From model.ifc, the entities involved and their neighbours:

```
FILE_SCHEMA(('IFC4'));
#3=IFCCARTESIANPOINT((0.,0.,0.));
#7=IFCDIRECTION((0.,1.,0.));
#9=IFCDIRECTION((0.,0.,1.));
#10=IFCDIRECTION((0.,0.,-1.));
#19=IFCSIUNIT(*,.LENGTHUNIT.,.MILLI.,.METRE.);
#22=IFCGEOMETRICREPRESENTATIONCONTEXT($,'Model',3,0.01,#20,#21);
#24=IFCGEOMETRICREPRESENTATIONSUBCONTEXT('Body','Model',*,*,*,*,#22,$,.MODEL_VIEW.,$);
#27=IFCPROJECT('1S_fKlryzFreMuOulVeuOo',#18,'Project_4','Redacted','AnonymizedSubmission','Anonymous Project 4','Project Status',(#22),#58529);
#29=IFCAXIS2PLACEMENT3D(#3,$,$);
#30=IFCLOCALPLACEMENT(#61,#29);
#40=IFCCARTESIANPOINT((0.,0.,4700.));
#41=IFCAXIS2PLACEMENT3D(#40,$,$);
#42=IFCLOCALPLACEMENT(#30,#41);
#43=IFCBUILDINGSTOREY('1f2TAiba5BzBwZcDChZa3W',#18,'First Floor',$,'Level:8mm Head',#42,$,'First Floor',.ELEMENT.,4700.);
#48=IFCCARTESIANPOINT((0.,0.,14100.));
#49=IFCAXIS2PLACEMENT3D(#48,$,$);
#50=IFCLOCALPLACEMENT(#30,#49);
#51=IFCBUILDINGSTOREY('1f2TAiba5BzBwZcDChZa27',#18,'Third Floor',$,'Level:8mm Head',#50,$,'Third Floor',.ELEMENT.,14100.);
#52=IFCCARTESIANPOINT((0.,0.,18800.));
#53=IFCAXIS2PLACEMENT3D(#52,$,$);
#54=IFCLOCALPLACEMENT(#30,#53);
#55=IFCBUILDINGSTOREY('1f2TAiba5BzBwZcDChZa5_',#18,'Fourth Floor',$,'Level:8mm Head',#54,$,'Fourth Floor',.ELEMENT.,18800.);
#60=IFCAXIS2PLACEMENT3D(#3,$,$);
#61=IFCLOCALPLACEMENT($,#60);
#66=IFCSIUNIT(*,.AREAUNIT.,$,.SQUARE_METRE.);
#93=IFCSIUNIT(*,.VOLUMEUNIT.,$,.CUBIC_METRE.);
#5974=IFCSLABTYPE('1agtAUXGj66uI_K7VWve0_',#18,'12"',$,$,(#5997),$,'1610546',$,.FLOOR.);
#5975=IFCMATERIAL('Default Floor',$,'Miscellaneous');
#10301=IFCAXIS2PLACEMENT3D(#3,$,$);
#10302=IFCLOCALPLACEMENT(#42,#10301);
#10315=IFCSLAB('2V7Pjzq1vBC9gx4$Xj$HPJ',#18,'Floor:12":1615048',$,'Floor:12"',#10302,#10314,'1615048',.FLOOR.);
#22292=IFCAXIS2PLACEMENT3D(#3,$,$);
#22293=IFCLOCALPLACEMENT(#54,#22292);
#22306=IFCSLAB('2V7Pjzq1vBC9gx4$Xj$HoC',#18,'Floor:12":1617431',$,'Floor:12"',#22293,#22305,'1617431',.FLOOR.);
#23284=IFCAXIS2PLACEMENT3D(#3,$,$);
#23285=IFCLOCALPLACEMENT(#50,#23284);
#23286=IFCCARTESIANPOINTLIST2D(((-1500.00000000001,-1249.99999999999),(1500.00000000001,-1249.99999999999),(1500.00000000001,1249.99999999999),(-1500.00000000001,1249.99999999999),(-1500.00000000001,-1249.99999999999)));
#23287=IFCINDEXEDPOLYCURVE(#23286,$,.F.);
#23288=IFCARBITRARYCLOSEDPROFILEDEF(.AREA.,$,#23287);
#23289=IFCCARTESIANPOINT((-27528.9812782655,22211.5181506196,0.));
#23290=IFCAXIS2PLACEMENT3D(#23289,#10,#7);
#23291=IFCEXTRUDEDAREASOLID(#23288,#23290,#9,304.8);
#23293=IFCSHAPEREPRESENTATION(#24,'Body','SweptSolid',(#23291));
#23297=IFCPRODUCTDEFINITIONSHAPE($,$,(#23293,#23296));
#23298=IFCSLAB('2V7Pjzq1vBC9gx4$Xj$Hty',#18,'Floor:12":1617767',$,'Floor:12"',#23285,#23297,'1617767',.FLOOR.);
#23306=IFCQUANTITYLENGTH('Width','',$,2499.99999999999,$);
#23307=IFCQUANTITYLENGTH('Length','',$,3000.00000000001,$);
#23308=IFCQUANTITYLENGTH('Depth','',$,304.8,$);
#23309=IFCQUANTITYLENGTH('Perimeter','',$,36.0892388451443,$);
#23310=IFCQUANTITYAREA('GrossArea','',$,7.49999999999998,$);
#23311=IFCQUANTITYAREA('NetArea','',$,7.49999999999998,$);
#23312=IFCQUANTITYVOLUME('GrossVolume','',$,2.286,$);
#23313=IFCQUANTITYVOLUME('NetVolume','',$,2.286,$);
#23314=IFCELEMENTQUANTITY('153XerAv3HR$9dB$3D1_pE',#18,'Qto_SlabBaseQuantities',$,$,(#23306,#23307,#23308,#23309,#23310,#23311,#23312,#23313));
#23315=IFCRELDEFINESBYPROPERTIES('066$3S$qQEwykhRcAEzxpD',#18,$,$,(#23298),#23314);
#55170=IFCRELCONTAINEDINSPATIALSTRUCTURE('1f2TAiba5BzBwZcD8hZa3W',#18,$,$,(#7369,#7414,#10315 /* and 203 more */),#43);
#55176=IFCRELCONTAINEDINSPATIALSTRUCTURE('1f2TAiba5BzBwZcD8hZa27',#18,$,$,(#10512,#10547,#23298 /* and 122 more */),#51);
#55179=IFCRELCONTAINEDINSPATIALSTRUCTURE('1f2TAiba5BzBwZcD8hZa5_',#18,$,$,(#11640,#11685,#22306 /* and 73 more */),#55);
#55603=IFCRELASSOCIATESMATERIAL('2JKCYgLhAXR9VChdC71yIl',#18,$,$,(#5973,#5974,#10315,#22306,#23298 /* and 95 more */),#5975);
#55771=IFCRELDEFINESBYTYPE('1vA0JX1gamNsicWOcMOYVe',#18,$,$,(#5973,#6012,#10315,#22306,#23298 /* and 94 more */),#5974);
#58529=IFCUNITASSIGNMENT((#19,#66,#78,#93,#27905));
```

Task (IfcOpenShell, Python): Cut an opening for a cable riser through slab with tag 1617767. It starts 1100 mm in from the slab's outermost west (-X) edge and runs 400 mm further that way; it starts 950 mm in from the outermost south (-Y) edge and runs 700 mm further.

```python
import numpy as np
import ifcopenshell
import ifcopenshell.api.feature
import ifcopenshell.api.geometry
import ifcopenshell.api.pset
import ifcopenshell.api.root
import ifcopenshell.geom
import ifcopenshell.util.element
import ifcopenshell.util.placement
import ifcopenshell.util.representation
import ifcopenshell.util.shape
import ifcopenshell.util.unit

model = ifcopenshell.open("model.ifc")
unit_scale = ifcopenshell.util.unit.calculate_unit_scale(model)
area_scale = ifcopenshell.util.unit.calculate_unit_scale(model, "AREAUNIT")
volume_scale = ifcopenshell.util.unit.calculate_unit_scale(model, "VOLUMEUNIT")
settings = ifcopenshell.geom.settings()


def volume(element):
    """Net volume in cubic metres, openings subtracted."""
    shape = ifcopenshell.geom.create_shape(settings, element)
    return ifcopenshell.util.shape.get_volume(shape.geometry)


slab = model.by_guid("2V7Pjzq1vBC9gx4$Xj$Hty")
before = volume(slab)

# Extent in the slab's own axes, in metres. The edges named are its -X and -Y sides.
slab_shape = ifcopenshell.geom.create_shape(settings, slab)
vertices = ifcopenshell.util.shape.get_vertices(slab_shape.geometry)
x_min, y_min, bottom = vertices.min(axis=0)
top = vertices[:, 2].max()

opening = ifcopenshell.api.root.create_entity(model, ifc_class="IfcOpeningElement", name="Cable riser opening", predefined_type="OPENING")
context = ifcopenshell.util.representation.get_context(model, "Model", "Body", "MODEL_VIEW")
width, depth = 0.4, 0.7
outline = [(0.0, 0.0), (width, 0.0), (width, depth), (0.0, depth), (0.0, 0.0)]
# Overshoot both faces by 50 mm so the cut is clean.
shape = ifcopenshell.api.geometry.add_slab_representation(
    model, context=context, depth=top - bottom + 0.1, polyline=outline
)
ifcopenshell.api.geometry.assign_representation(model, product=opening, representation=shape)

matrix = ifcopenshell.util.placement.get_local_placement(slab.ObjectPlacement)
matrix[:, 3] = matrix @ np.append(np.array([x_min + 1.1, y_min + 0.95, bottom - 0.05]) / unit_scale, 1.0)
ifcopenshell.api.geometry.edit_object_placement(model, product=opening, matrix=matrix, is_si=False)
ifcopenshell.api.feature.add_feature(model, feature=opening, element=slab)

after = volume(slab)

# Update the slab's stored quantities.
qto = model.by_id(ifcopenshell.util.element.get_pset(slab, "Qto_SlabBaseQuantities", should_inherit=False)["id"])
ifcopenshell.api.pset.edit_qto(model, qto=qto, properties={
    "NetArea": after / (top - bottom) / area_scale,
    "NetVolume": after / volume_scale,
})

print(f"slab volume {before:.3f} -> {after:.3f} m3")

model.write("model_v2.ifc")
```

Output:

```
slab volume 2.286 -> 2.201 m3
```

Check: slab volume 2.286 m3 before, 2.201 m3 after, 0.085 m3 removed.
